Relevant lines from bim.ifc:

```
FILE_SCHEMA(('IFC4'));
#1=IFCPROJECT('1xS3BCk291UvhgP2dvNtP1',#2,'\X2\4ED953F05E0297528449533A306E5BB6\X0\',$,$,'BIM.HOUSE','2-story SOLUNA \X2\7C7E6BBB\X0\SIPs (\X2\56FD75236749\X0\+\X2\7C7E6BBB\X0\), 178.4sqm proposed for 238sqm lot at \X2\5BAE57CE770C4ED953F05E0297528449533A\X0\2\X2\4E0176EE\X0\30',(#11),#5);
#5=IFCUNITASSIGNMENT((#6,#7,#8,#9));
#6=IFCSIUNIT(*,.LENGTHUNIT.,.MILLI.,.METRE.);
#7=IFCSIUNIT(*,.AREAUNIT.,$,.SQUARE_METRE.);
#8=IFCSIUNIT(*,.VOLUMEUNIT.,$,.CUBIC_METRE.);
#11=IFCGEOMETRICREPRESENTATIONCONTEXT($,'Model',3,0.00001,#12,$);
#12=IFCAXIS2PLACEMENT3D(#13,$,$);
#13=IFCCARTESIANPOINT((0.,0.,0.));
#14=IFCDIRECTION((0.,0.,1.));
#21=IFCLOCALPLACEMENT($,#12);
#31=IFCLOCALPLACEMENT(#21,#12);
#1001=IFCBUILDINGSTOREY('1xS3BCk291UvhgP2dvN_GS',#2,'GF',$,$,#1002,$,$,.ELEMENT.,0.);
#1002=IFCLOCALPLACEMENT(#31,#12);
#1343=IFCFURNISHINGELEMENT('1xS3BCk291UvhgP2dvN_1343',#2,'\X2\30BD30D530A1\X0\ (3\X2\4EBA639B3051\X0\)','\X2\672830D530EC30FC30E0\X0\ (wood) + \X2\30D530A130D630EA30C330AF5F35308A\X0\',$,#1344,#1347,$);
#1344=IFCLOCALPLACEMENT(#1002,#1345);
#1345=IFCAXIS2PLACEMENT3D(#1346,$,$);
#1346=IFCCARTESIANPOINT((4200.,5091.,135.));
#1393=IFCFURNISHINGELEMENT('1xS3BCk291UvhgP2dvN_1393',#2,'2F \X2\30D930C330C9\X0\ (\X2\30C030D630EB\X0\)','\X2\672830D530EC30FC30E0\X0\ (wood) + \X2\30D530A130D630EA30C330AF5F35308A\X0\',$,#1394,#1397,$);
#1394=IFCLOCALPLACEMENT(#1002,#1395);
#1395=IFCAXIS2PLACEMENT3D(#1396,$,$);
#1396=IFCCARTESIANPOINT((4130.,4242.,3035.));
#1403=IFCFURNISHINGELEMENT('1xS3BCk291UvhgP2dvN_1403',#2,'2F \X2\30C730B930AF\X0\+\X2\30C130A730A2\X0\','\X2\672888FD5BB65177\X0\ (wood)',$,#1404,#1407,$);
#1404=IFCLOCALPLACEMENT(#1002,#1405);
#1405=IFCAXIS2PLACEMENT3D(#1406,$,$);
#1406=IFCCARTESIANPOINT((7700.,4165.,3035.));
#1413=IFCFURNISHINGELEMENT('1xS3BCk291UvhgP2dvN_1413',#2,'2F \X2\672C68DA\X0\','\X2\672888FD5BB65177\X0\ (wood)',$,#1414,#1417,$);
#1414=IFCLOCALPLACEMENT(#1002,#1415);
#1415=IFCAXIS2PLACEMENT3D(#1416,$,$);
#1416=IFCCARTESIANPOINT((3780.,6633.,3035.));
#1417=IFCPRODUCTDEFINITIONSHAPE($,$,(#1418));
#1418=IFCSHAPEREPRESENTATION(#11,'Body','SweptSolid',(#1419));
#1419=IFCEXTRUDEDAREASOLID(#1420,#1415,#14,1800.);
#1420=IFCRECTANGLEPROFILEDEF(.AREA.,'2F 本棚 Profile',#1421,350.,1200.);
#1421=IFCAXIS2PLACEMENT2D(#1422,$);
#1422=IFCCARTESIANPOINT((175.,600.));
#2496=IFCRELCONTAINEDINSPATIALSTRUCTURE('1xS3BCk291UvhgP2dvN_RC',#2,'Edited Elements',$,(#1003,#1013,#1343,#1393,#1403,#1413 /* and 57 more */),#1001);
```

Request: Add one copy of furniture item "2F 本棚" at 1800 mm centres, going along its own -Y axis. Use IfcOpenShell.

```python
import ifcopenshell
import ifcopenshell.api.geometry
import ifcopenshell.api.root
import ifcopenshell.util.element
import ifcopenshell.util.placement
import ifcopenshell.util.unit

model = ifcopenshell.open("bim.ifc")
unit_scale = ifcopenshell.util.unit.calculate_unit_scale(model)


def reuse_history(source, copy):
    """copy_class also copies each property set's owner history, people and application; keep the originals."""
    for rel in copy.IsDefinedBy:
        if rel.is_a("IfcRelDefinesByProperties") and (history := rel.RelatingPropertyDefinition.OwnerHistory):
            rel.RelatingPropertyDefinition.OwnerHistory = source.OwnerHistory
            ifcopenshell.util.element.remove_deep2(model, history)


source = model.by_id(1413)
base = ifcopenshell.util.placement.get_local_placement(source.ObjectPlacement)
step = -base[:3, 1] * 1.8 / unit_scale

for i in range(1, 2):
    copy = ifcopenshell.api.root.copy_class(model, product=source)
    copy.Representation = ifcopenshell.util.element.copy_deep(
        model, source.Representation, exclude=["IfcGeometricRepresentationContext", "IfcRepresentationMap"]
    )
    reuse_history(source, copy)
    matrix = base.copy()
    matrix[:3, 3] += i * step
    print("added at", matrix[:3, 3].round(3) + 0.0)
    ifcopenshell.api.geometry.edit_object_placement(model, product=copy, matrix=matrix, is_si=False)

model.write("bim_rev.ifc")
```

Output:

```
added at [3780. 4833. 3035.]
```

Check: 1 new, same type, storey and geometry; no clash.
